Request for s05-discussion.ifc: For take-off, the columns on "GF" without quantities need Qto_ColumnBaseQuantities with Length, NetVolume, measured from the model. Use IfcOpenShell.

First a look at what the model holds.

```python
import ifcopenshell
import ifcopenshell.util.element
import ifcopenshell.util.unit

model = ifcopenshell.open("s05-discussion.ifc")
print(model.schema)
for unit_type in ("LENGTHUNIT", "AREAUNIT", "VOLUMEUNIT"):
    print(unit_type, ifcopenshell.util.unit.calculate_unit_scale(model, unit_type))
storey = next(s for s in model.by_type("IfcBuildingStorey") if s.Name == "GF")
columns = [e for e in ifcopenshell.util.element.get_decomposition(storey) if e.is_a("IfcColumn")]
for e in sorted(columns, key=lambda e: e.id()):
    print(e.id(), e.is_a(), e.Name, list(ifcopenshell.util.element.get_psets(e, qtos_only=True)), sep=" | ")
```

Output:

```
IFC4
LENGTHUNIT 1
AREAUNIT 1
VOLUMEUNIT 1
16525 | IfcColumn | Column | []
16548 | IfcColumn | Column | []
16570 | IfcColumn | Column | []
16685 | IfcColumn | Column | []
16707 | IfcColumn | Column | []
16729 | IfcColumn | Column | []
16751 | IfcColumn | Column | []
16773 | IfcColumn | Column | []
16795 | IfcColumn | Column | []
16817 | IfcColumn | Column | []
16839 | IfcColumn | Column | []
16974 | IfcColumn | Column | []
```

```python
import ifcopenshell
import ifcopenshell.api.pset
import ifcopenshell.geom
import ifcopenshell.util.element
import ifcopenshell.util.shape
import ifcopenshell.util.unit

model = ifcopenshell.open("s05-discussion.ifc")
unit_scale = ifcopenshell.util.unit.calculate_unit_scale(model)
volume_scale = ifcopenshell.util.unit.calculate_unit_scale(model, "VOLUMEUNIT")
settings = ifcopenshell.geom.settings()

storey = next(s for s in model.by_type("IfcBuildingStorey") if s.Name == "GF")
columns = [e for e in ifcopenshell.util.element.get_decomposition(storey) if e.is_a("IfcColumn")]

for e in sorted(columns, key=lambda e: e.id()):
    if ifcopenshell.util.element.get_psets(e, qtos_only=True, should_inherit=False):
        continue
    # Geometry comes back in metres, in the element's own axes.
    shape = ifcopenshell.geom.create_shape(settings, e)
    values = {
        "Length": ifcopenshell.util.shape.get_z(shape.geometry) / unit_scale,
        "NetVolume": ifcopenshell.util.shape.get_volume(shape.geometry) / volume_scale,
    }
    qto = ifcopenshell.api.pset.add_qto(model, product=e, name="Qto_ColumnBaseQuantities")
    ifcopenshell.api.pset.edit_qto(model, qto=qto, properties=values)
    print(e.id(), {k: round(v, 3) for k, v in values.items()})

model.write("s05-discussion_rev.ifc")
```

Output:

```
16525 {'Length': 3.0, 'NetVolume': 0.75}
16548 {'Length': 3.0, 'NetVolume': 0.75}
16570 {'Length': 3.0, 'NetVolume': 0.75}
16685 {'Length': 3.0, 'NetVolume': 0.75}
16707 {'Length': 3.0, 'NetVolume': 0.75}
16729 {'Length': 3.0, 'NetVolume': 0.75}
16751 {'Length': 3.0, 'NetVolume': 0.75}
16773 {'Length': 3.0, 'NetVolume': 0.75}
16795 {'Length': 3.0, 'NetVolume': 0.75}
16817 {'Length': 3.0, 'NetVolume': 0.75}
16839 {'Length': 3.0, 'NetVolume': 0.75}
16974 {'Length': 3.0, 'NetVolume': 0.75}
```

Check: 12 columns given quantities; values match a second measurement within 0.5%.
